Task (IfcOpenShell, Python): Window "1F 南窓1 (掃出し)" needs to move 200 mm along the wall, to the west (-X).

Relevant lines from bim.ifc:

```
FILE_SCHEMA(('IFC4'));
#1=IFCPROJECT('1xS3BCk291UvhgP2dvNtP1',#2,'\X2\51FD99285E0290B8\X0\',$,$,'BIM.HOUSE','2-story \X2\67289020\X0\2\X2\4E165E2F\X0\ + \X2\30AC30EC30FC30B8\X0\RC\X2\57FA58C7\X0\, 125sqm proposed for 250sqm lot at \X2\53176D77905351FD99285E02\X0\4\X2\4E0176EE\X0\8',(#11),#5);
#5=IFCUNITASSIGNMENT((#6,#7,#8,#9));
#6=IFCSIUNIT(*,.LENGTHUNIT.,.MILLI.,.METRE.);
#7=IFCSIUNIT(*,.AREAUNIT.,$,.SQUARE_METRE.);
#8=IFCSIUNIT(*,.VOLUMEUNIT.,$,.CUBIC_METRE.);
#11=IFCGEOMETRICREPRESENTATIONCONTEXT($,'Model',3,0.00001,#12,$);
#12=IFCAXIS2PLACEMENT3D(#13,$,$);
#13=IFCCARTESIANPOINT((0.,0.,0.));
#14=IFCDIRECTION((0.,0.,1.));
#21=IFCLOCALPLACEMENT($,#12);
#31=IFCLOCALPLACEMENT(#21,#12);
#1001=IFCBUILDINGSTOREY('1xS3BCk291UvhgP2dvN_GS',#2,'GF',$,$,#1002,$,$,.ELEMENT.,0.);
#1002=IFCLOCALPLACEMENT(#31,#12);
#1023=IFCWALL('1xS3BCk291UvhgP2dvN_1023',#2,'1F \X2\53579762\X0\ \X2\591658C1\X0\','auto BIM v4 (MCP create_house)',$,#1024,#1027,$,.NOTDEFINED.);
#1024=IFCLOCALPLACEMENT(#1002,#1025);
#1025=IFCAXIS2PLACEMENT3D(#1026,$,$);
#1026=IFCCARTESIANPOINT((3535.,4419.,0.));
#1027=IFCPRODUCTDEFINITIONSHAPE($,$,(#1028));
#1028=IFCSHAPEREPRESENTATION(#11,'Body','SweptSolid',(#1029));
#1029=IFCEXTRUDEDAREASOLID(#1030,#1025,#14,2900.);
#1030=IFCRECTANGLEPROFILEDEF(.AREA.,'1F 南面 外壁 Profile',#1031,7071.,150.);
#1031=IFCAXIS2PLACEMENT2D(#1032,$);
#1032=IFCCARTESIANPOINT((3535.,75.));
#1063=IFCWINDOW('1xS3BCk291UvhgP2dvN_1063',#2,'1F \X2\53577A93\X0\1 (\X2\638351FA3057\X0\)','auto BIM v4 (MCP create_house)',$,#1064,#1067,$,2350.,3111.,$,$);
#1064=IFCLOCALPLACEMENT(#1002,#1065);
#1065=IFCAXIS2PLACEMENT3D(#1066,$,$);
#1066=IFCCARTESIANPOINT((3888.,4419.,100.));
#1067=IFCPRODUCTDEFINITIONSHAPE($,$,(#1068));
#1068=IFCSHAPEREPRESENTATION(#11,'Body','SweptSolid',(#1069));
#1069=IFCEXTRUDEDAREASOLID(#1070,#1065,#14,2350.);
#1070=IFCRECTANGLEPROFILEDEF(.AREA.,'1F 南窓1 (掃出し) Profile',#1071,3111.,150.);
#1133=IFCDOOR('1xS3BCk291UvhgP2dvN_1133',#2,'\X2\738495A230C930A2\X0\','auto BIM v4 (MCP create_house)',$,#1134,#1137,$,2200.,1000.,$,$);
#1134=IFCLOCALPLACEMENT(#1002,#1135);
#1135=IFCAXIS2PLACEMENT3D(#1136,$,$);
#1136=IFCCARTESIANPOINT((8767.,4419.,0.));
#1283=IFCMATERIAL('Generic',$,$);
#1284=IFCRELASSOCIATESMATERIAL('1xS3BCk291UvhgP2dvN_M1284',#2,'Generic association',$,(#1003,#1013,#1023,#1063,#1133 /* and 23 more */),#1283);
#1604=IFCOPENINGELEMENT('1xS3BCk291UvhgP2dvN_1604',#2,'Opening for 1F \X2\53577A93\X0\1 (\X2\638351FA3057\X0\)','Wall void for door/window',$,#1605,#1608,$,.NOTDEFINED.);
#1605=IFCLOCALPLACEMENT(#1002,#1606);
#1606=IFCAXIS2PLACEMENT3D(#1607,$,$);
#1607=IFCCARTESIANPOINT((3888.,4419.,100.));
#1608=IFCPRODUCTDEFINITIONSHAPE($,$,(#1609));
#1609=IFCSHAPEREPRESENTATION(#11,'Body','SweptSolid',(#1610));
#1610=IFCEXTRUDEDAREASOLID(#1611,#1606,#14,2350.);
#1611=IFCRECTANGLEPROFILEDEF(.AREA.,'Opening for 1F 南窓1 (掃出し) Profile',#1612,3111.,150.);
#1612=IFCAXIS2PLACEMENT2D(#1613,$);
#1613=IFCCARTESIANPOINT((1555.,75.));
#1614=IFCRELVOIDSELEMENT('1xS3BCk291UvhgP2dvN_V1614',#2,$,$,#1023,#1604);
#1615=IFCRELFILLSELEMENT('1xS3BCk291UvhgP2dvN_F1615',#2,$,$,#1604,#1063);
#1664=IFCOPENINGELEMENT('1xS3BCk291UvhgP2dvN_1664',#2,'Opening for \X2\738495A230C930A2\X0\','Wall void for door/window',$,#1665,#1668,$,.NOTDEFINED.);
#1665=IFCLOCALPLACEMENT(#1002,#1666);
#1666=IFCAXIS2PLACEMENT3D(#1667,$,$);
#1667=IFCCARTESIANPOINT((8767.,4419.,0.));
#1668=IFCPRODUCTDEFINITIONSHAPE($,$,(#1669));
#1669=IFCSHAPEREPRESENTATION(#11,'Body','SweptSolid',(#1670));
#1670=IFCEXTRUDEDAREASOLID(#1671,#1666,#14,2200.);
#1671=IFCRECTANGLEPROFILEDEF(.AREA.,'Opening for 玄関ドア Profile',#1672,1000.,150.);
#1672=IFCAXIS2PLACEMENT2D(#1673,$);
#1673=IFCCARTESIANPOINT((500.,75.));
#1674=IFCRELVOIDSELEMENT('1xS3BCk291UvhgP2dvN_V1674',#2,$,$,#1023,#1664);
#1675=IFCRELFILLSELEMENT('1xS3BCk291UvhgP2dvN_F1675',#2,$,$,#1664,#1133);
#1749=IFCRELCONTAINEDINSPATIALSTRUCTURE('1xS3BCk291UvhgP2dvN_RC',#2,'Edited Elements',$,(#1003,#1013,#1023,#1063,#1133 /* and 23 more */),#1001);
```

```python
import ifcopenshell
import ifcopenshell.api.geometry
import ifcopenshell.util.placement
import ifcopenshell.util.unit

model = ifcopenshell.open("bim.ifc")
unit_scale = ifcopenshell.util.unit.calculate_unit_scale(model)

window = model.by_id(1063)
opening = window.FillsVoids[0].RelatingOpeningElement
wall = opening.VoidsElements[0].RelatingBuildingElement

wall_matrix = ifcopenshell.util.placement.get_local_placement(wall.ObjectPlacement)
shift = wall_matrix[:3, 0] * -0.2 / unit_scale
before = ifcopenshell.util.placement.get_local_placement(window.ObjectPlacement)[:3, 3].copy()

# The window is not placed relative to its opening, so move both.
for product in (opening, window):
    matrix = ifcopenshell.util.placement.get_local_placement(product.ObjectPlacement)
    matrix[:3, 3] += shift
    ifcopenshell.api.geometry.edit_object_placement(model, product=product, matrix=matrix, is_si=False)

after = ifcopenshell.util.placement.get_local_placement(window.ObjectPlacement)[:3, 3]
print("window moved by", (after - before).round(3) + 0.0)

model.write("bim_rev.ifc")
```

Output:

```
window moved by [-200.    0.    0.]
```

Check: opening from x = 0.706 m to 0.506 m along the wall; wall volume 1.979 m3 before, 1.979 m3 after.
